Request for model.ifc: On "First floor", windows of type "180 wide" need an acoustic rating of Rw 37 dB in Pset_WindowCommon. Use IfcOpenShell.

First a look at what the model holds.

```python
import ifcopenshell
import ifcopenshell.util.element

model = ifcopenshell.open("model.ifc")
print(model.schema)
storey = next(s for s in model.by_type("IfcBuildingStorey") if s.Name == "First floor")
windows = [e for e in ifcopenshell.util.element.get_decomposition(storey) if e.is_a("IfcWindow")]
seen = {}
for e in windows:
    element_type = ifcopenshell.util.element.get_type(e)
    key = (element_type.Name if element_type != e and element_type else None, ifcopenshell.util.element.get_pset(e, "Pset_WindowCommon", "AcousticRating"))
    seen[key] = seen.get(key, 0) + 1
for (name, value), count in sorted(seen.items(), key=str):
    print(count, "x", name, "|", value)
```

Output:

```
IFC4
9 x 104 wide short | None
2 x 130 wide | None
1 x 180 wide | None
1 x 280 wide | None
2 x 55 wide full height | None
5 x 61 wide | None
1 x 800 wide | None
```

```python
import ifcopenshell
import ifcopenshell.api.pset
import ifcopenshell.util.element

model = ifcopenshell.open("model.ifc")

storey = next(s for s in model.by_type("IfcBuildingStorey") if s.Name == "First floor")
windows = [e for e in ifcopenshell.util.element.get_decomposition(storey) if e.is_a("IfcWindow")]

count = 0
for e in windows:
    element_type = ifcopenshell.util.element.get_type(e)
    if element_type in (None, e) or element_type.Name != "180 wide":
        continue
    # add_pset returns the element's existing set when there is one.
    pset = ifcopenshell.api.pset.add_pset(model, product=e, name="Pset_WindowCommon")
    ifcopenshell.api.pset.edit_pset(model, pset=pset, properties={"AcousticRating": "Rw 37 dB"})
    count += 1

print(count, "windows updated")

model.write("model_updated.ifc")
```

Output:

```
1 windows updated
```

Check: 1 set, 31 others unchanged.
